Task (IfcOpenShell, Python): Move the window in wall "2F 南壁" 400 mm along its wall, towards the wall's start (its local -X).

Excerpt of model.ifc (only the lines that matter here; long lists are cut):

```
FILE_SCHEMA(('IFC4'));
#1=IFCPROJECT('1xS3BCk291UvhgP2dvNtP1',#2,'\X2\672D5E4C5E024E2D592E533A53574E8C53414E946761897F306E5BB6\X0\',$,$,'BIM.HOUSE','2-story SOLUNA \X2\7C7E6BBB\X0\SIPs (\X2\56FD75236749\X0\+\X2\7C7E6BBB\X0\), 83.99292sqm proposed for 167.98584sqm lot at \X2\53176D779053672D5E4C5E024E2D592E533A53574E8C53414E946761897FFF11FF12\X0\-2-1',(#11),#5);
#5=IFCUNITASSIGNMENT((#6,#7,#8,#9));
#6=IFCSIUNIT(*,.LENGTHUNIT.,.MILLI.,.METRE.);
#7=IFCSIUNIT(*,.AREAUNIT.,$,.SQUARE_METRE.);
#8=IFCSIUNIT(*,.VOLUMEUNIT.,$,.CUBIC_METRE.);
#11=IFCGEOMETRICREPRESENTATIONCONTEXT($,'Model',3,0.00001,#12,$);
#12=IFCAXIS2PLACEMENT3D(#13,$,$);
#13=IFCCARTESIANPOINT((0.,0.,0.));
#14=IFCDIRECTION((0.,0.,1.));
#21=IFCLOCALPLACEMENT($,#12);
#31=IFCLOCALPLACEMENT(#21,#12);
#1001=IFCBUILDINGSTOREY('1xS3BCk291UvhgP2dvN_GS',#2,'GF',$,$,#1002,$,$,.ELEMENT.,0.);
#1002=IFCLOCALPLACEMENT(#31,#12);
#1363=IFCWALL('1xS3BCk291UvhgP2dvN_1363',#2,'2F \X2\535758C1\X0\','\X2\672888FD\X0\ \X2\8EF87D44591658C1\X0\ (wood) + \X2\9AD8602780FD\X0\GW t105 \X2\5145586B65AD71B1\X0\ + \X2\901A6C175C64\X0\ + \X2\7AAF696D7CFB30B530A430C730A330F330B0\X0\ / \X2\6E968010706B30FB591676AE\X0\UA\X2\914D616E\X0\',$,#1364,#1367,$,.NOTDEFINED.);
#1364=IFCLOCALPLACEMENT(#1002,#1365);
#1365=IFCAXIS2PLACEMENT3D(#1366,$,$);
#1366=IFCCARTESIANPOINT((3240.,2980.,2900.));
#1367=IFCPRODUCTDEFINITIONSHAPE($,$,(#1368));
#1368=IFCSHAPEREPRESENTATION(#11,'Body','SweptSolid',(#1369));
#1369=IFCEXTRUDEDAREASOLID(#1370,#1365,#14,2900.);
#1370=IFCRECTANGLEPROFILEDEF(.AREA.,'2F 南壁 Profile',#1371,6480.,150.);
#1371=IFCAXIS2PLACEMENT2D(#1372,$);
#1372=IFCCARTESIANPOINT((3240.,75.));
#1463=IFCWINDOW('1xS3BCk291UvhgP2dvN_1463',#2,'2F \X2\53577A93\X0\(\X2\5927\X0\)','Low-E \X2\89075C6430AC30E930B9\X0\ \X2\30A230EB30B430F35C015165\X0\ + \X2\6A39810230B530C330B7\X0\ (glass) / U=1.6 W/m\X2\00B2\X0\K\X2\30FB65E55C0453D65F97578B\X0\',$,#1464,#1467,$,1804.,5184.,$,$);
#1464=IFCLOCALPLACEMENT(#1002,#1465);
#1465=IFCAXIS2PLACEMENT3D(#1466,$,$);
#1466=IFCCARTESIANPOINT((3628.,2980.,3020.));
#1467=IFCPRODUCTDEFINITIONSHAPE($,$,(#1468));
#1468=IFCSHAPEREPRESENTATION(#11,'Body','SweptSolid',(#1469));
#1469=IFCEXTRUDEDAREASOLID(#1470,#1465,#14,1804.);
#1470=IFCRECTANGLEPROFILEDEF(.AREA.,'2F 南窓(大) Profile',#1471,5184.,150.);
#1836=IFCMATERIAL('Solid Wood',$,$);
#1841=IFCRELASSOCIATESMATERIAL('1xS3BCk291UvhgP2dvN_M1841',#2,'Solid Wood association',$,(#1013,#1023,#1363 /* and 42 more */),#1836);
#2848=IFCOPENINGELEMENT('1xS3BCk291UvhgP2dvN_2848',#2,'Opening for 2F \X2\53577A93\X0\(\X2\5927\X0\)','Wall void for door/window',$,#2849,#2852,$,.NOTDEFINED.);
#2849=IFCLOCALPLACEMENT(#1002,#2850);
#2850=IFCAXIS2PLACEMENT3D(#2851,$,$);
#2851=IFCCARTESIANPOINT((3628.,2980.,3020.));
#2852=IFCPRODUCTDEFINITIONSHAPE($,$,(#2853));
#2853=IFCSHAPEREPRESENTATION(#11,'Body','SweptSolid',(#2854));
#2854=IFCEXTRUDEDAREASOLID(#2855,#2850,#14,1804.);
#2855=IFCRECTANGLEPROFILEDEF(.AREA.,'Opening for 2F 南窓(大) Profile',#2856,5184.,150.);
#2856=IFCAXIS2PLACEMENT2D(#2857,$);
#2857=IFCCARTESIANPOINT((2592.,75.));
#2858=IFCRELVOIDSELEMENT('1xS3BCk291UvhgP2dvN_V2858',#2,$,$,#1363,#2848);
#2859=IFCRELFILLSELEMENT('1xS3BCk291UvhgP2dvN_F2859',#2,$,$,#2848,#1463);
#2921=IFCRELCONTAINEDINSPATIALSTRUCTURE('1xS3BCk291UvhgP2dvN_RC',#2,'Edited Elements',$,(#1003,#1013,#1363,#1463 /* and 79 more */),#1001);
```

```python
import ifcopenshell
import ifcopenshell.api.geometry
import ifcopenshell.util.placement
import ifcopenshell.util.unit

model = ifcopenshell.open("model.ifc")
unit_scale = ifcopenshell.util.unit.calculate_unit_scale(model)

window = model.by_id(1463)
opening = window.FillsVoids[0].RelatingOpeningElement
wall = opening.VoidsElements[0].RelatingBuildingElement

wall_matrix = ifcopenshell.util.placement.get_local_placement(wall.ObjectPlacement)
shift = wall_matrix[:3, 0] * -0.4 / unit_scale
before = ifcopenshell.util.placement.get_local_placement(window.ObjectPlacement)[:3, 3].copy()

# The window is not placed relative to its opening, so move both.
for product in (opening, window):
    matrix = ifcopenshell.util.placement.get_local_placement(product.ObjectPlacement)
    matrix[:3, 3] += shift
    ifcopenshell.api.geometry.edit_object_placement(model, product=product, matrix=matrix, is_si=False)

after = ifcopenshell.util.placement.get_local_placement(window.ObjectPlacement)[:3, 3]
print("window moved by", (after - before).round(3) + 0.0)

model.write("model_v2.ifc")
```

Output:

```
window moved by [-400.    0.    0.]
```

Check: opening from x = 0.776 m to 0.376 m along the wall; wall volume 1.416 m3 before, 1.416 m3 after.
